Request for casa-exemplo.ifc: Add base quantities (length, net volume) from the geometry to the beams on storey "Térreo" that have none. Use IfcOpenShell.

First a look at what the model holds.

```python
import ifcopenshell
import ifcopenshell.util.element
import ifcopenshell.util.unit

model = ifcopenshell.open("casa-exemplo.ifc")
print(model.schema)
for unit_type in ("LENGTHUNIT", "AREAUNIT", "VOLUMEUNIT"):
    print(unit_type, ifcopenshell.util.unit.calculate_unit_scale(model, unit_type))
storey = next(s for s in model.by_type("IfcBuildingStorey") if s.Name == "Térreo")
beams = [e for e in ifcopenshell.util.element.get_decomposition(storey) if e.is_a("IfcBeam")]
for e in sorted(beams, key=lambda e: e.id()):
    print(e.id(), e.is_a(), e.Name, list(ifcopenshell.util.element.get_psets(e, qtos_only=True)), sep=" | ")
```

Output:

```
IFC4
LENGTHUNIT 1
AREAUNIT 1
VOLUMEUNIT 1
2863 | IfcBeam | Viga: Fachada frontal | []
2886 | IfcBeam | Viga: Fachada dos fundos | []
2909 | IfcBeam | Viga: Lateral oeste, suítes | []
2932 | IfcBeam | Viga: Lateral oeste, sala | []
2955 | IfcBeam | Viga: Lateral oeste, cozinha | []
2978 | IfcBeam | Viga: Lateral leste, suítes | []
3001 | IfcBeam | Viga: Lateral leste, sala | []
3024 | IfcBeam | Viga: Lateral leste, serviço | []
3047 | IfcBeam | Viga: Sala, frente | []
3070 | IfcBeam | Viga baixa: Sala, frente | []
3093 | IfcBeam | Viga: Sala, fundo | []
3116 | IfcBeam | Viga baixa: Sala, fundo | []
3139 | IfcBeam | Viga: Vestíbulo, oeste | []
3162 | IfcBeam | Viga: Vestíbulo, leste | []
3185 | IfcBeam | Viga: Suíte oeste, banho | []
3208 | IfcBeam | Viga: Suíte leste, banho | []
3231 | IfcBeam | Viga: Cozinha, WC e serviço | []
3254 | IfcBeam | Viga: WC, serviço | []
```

```python
import ifcopenshell
import ifcopenshell.api.pset
import ifcopenshell.geom
import ifcopenshell.util.element
import ifcopenshell.util.shape
import ifcopenshell.util.unit

model = ifcopenshell.open("casa-exemplo.ifc")
unit_scale = ifcopenshell.util.unit.calculate_unit_scale(model)
volume_scale = ifcopenshell.util.unit.calculate_unit_scale(model, "VOLUMEUNIT")
settings = ifcopenshell.geom.settings()

storey = next(s for s in model.by_type("IfcBuildingStorey") if s.Name == "Térreo")
beams = [e for e in ifcopenshell.util.element.get_decomposition(storey) if e.is_a("IfcBeam")]

for e in sorted(beams, key=lambda e: e.id()):
    if ifcopenshell.util.element.get_psets(e, qtos_only=True, should_inherit=False):
        continue
    # Geometry comes back in metres, in the element's own axes.
    shape = ifcopenshell.geom.create_shape(settings, e)
    values = {
        "Length": ifcopenshell.util.shape.get_max_xyz(shape.geometry) / unit_scale,
        "NetVolume": ifcopenshell.util.shape.get_volume(shape.geometry) / volume_scale,
    }
    qto = ifcopenshell.api.pset.add_qto(model, product=e, name="Qto_BeamBaseQuantities")
    ifcopenshell.api.pset.edit_qto(model, qto=qto, properties=values)
    print(e.id(), {k: round(v, 3) for k, v in values.items()})

model.write("casa-exemplo_edited.ifc")
```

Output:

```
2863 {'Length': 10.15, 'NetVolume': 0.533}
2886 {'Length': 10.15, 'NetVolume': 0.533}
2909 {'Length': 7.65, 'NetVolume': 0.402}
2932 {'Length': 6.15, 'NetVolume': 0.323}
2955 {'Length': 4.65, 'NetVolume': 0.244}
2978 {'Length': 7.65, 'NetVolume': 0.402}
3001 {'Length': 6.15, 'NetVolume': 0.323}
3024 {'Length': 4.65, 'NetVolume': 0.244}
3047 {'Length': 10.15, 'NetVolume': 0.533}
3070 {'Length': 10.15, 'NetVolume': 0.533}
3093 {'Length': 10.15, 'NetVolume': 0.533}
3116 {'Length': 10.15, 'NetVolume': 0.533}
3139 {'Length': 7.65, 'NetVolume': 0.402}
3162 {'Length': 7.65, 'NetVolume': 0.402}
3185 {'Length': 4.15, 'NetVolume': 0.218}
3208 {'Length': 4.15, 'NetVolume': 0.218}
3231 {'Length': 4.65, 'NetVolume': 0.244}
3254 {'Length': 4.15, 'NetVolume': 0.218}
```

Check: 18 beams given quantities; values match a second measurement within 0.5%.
